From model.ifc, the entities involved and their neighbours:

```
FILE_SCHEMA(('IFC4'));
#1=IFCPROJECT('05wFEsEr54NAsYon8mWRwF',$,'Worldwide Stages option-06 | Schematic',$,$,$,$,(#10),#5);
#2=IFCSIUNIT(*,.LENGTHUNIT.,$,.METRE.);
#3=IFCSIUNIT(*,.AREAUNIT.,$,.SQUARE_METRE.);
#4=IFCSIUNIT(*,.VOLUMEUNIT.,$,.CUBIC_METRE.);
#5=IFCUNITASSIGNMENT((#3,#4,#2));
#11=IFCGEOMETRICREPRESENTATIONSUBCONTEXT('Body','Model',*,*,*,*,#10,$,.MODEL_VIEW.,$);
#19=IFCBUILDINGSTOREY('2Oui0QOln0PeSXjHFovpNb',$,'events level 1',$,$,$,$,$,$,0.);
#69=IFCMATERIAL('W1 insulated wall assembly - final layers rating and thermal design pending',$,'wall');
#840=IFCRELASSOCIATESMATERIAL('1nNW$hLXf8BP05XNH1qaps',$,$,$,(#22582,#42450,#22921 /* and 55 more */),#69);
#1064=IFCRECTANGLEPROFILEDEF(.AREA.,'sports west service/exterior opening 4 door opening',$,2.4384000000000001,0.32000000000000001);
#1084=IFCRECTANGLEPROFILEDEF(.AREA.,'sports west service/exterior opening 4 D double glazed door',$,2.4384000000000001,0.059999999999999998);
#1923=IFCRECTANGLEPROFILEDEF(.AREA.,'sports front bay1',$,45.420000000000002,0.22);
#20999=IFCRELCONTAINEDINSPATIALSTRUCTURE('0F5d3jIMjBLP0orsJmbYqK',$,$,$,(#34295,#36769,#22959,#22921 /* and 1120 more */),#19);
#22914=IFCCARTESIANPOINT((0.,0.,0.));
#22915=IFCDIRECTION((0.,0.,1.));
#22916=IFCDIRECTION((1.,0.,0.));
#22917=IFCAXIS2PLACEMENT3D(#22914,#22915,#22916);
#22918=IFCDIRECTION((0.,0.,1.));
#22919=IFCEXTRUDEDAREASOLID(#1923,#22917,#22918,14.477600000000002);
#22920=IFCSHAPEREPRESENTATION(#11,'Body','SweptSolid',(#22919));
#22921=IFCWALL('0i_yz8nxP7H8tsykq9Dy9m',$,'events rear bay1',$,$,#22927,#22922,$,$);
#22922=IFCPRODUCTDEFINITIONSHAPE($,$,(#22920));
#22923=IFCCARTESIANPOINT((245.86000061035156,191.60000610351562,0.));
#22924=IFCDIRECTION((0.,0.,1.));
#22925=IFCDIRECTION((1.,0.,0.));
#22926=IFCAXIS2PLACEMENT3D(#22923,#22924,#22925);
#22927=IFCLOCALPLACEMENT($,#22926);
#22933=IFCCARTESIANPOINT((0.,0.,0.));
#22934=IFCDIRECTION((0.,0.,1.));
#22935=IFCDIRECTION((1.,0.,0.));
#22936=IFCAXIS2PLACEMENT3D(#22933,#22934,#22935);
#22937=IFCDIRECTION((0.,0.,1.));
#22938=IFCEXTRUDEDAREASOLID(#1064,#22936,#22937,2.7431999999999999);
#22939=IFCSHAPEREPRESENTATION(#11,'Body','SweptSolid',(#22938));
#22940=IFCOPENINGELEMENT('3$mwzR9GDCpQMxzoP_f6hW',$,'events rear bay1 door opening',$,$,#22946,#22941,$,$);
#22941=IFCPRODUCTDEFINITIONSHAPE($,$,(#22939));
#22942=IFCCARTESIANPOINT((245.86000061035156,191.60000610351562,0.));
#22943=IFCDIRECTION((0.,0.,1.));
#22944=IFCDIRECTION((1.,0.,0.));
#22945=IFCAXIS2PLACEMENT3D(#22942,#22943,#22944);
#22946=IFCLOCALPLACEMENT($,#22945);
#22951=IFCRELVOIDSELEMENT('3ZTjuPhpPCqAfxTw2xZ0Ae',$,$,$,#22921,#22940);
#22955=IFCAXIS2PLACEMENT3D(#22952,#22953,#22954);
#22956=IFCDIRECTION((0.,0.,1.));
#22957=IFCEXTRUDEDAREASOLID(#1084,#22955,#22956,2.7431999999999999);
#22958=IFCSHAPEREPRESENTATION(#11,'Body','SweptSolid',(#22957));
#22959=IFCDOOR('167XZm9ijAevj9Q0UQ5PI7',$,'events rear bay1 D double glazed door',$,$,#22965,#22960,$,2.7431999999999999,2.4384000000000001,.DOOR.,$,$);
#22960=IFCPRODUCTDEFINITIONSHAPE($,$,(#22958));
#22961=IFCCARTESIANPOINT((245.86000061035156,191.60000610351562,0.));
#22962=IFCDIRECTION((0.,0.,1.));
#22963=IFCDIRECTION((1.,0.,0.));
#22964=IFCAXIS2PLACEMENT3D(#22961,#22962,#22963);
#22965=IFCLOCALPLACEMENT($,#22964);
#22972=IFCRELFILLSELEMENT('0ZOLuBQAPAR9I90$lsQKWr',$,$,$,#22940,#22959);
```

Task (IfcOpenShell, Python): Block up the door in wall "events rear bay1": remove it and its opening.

```python
import ifcopenshell
import ifcopenshell.api.feature
import ifcopenshell.api.root
import ifcopenshell.geom
import ifcopenshell.util.shape

model = ifcopenshell.open("model.ifc")
settings = ifcopenshell.geom.settings()


def volume(element):
    """Net volume in cubic metres, openings subtracted."""
    shape = ifcopenshell.geom.create_shape(settings, element)
    return ifcopenshell.util.shape.get_volume(shape.geometry)


door = model.by_id(22959)
opening = door.FillsVoids[0].RelatingOpeningElement
wall = opening.VoidsElements[0].RelatingBuildingElement
before = volume(wall)

ifcopenshell.api.root.remove_product(model, product=door)
ifcopenshell.api.feature.remove_feature(model, feature=opening)

after = volume(wall)

print(f"wall volume {before:.3f} -> {after:.3f} m3")

model.write("model-out.ifc")
```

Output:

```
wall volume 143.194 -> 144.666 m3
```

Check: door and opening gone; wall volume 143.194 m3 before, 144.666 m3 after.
